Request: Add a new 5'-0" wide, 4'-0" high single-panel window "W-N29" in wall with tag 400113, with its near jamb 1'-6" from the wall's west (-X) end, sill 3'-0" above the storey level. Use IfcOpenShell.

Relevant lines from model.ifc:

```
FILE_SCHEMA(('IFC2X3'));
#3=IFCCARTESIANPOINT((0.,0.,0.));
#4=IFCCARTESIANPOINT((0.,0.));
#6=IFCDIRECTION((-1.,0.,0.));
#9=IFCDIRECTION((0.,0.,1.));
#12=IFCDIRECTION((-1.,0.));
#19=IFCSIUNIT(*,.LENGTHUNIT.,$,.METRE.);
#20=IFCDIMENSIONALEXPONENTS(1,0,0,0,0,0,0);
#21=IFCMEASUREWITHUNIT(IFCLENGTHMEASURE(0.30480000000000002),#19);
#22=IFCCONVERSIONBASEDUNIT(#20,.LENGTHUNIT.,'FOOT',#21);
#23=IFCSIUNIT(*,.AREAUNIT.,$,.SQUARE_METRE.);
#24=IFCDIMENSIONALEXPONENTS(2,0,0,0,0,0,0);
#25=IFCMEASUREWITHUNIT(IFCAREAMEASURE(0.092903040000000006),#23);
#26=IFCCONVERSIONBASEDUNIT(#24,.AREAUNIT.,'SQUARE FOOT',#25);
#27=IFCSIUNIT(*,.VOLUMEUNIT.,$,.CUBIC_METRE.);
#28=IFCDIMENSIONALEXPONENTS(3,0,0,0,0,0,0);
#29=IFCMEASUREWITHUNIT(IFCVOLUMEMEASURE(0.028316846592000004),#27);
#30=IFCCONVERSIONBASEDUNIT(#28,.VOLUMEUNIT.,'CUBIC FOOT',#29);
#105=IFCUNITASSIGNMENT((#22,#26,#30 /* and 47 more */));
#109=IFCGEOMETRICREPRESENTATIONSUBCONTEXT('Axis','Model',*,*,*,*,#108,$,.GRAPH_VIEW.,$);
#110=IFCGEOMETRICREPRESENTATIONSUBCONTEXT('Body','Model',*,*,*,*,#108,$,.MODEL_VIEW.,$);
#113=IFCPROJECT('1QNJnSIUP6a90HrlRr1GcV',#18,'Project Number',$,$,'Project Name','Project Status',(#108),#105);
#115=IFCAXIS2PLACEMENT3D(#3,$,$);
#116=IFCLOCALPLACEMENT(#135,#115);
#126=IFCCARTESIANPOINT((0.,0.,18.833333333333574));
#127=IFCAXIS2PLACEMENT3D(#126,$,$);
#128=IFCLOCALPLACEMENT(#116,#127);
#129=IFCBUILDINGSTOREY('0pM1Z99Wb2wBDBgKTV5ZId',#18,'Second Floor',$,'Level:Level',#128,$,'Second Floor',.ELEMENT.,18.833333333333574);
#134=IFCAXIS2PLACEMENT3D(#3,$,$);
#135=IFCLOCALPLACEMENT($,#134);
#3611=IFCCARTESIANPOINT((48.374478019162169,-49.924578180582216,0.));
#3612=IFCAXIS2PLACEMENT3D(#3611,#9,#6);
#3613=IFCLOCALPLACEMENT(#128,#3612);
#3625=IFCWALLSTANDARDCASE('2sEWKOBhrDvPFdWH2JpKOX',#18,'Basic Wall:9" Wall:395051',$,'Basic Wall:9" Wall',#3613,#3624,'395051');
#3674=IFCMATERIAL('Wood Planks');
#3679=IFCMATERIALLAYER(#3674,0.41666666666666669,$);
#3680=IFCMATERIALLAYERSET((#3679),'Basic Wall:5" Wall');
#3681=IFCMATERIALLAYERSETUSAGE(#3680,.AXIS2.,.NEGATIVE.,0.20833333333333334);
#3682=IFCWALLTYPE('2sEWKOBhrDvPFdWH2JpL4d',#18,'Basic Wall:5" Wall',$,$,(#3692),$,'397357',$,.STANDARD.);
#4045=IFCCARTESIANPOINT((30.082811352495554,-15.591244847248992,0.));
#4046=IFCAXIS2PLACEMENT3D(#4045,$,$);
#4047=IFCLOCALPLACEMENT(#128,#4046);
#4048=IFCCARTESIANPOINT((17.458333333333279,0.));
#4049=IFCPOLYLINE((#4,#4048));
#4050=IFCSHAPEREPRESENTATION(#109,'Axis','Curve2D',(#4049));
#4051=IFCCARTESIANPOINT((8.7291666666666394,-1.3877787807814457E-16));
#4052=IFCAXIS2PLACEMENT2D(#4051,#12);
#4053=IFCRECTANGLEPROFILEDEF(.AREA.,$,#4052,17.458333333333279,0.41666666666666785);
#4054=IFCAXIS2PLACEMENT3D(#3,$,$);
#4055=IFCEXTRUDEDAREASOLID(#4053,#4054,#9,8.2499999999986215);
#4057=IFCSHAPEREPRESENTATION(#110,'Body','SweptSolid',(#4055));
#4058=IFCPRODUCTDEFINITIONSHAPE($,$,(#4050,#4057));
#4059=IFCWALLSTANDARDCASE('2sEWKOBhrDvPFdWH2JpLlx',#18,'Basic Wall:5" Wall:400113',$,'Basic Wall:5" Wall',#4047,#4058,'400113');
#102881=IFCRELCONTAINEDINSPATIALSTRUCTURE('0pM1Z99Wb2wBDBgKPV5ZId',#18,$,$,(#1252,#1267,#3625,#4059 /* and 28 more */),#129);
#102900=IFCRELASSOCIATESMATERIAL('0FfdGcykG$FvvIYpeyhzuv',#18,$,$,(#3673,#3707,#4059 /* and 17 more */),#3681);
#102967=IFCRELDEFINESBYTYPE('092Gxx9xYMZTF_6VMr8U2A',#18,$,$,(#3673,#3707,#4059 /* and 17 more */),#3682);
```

```python
import numpy as np
import ifcopenshell
import ifcopenshell.api.feature
import ifcopenshell.api.geometry
import ifcopenshell.api.root
import ifcopenshell.api.spatial
import ifcopenshell.api.type
import ifcopenshell.geom
import ifcopenshell.util.element
import ifcopenshell.util.placement
import ifcopenshell.util.representation
import ifcopenshell.util.shape
import ifcopenshell.util.unit

model = ifcopenshell.open("model.ifc")
unit_scale = ifcopenshell.util.unit.calculate_unit_scale(model)
settings = ifcopenshell.geom.settings()


def volume(element):
    """Net volume in cubic metres, openings subtracted."""
    shape = ifcopenshell.geom.create_shape(settings, element)
    return ifcopenshell.util.shape.get_volume(shape.geometry)


wall = model.by_guid("2sEWKOBhrDvPFdWH2JpLlx")
storey = ifcopenshell.util.element.get_container(wall, ifc_class="IfcBuildingStorey")
context = ifcopenshell.util.representation.get_context(model, "Model", "Body", "MODEL_VIEW")
before = volume(wall)

width, height, from_end, sill = 1.524, 1.2192, 0.4572, 0.9144  # metres

# The wall runs along its own X axis, and the end named is its -X end.
wall_shape = ifcopenshell.geom.create_shape(settings, wall)
x, y, z = ifcopenshell.util.shape.get_vertices(wall_shape.geometry).T
start = x.min() + from_end
face, thickness = float(y.min()), float(y.max() - y.min())
wall_matrix = ifcopenshell.util.placement.get_local_placement(wall.ObjectPlacement)
level = ifcopenshell.util.placement.get_local_placement(storey.ObjectPlacement)[2, 3]


def in_wall(x, y):
    """Placement at x, y metres in the wall's axes, at sill height."""
    matrix = wall_matrix.copy()
    matrix[:, 3] = wall_matrix @ np.array([x / unit_scale, y / unit_scale, 0.0, 1.0])
    matrix[2, 3] = level + sill / unit_scale
    return matrix


# Opening: a box that overshoots both wall faces by 50 mm.
opening = ifcopenshell.api.root.create_entity(model, ifc_class="IfcOpeningElement")
box = ifcopenshell.api.geometry.add_wall_representation(
    model, context=context, length=width, height=height, thickness=thickness + 0.1
)
ifcopenshell.api.geometry.assign_representation(model, product=opening, representation=box)
ifcopenshell.api.geometry.edit_object_placement(model, product=opening, matrix=in_wall(start, face - 0.05), is_si=False)
ifcopenshell.api.feature.add_feature(model, feature=opening, element=wall)

window = ifcopenshell.api.root.create_entity(model, ifc_class="IfcWindow", name="W-N29")
window.OverallWidth, window.OverallHeight = width / unit_scale, height / unit_scale
body = ifcopenshell.api.geometry.add_window_representation(
    model,
    context=context,
    overall_width=window.OverallWidth,
    overall_height=window.OverallHeight,
    partition_type="SINGLE_PANEL",
)
ifcopenshell.api.geometry.assign_representation(model, product=window, representation=body)
ifcopenshell.api.spatial.assign_container(model, products=[window], relating_structure=storey)
fills = ifcopenshell.api.feature.add_filling(model, opening=opening, element=window)
fills.OwnerHistory = window.OwnerHistory  # required in IFC2X3

# IFC2X3 keeps the operation on the window style.
style = ifcopenshell.api.root.create_entity(model, ifc_class="IfcWindowStyle", name="W-N29")
style.OperationType, style.ConstructionType = "SINGLE_PANEL", "NOTDEFINED"
style.ParameterTakesPrecedence = style.Sizeable = False
ifcopenshell.api.type.assign_type(model, related_objects=[window], relating_type=style)

# Centre the window in the wall's thickness.
ifcopenshell.api.geometry.edit_object_placement(model, product=window, matrix=in_wall(start, face), is_si=False)
window_shape = ifcopenshell.geom.create_shape(settings, window)
depth = ifcopenshell.util.shape.get_vertices(window_shape.geometry)[:, 1]
offset = face + thickness / 2 - (depth.min() + depth.max()) / 2
ifcopenshell.api.geometry.edit_object_placement(model, product=window, matrix=in_wall(start, offset), is_si=False)

after = volume(wall)

print(f"wall volume {before:.3f} -> {after:.3f} m3")

model.write("model_v2.ifc")
```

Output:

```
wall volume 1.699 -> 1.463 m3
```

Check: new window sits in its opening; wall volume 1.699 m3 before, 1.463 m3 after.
